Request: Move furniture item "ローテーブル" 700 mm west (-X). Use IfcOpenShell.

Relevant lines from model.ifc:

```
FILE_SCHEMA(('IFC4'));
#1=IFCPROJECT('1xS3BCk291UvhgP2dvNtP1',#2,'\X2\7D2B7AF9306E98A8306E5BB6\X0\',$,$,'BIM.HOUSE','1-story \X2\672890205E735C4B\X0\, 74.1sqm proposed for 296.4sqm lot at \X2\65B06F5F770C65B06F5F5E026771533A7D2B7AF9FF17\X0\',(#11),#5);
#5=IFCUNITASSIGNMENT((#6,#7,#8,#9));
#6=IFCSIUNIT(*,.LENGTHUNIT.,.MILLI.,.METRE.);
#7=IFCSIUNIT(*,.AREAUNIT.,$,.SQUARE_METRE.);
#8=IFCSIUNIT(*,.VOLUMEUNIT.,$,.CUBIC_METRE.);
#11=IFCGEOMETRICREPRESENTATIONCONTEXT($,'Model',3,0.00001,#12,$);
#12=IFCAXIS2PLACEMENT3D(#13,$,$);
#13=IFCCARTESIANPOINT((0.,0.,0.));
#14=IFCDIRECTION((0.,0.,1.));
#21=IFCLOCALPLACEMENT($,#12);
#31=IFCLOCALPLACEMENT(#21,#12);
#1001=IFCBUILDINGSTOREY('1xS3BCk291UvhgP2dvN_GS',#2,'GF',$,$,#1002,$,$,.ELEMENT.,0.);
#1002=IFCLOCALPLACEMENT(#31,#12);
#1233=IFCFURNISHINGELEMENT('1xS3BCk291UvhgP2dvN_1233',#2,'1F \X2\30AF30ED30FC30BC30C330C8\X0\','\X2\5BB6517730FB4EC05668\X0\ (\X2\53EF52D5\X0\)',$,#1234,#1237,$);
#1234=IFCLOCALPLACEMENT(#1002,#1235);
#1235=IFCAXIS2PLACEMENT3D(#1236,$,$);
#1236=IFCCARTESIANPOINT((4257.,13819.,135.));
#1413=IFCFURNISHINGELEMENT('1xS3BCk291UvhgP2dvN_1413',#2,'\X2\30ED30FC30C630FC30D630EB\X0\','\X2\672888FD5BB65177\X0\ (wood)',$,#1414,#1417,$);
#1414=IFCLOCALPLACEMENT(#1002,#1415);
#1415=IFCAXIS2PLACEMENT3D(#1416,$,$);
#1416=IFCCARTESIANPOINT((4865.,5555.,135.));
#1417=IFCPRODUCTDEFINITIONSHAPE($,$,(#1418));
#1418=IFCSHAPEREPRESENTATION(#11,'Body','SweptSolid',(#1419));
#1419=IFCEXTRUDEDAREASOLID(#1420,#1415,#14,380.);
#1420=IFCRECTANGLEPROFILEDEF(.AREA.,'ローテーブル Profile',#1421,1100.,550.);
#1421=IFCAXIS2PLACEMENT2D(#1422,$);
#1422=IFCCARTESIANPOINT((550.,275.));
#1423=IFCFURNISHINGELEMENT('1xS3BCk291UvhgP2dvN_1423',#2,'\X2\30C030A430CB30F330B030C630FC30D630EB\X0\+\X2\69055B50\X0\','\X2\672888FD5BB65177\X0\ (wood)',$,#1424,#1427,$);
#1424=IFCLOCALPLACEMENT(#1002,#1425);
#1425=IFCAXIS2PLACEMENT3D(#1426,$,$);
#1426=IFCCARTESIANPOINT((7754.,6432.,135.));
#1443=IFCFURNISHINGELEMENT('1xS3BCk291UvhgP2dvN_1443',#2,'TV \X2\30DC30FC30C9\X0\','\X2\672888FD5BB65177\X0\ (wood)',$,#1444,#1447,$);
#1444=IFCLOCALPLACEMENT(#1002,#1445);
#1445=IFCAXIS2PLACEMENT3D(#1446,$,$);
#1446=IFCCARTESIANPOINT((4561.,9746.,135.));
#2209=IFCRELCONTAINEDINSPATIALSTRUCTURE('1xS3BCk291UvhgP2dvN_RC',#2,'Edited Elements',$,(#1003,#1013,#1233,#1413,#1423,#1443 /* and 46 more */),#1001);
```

```python
import ifcopenshell
import ifcopenshell.api.geometry
import ifcopenshell.util.placement
import ifcopenshell.util.unit

model = ifcopenshell.open("model.ifc")
unit_scale = ifcopenshell.util.unit.calculate_unit_scale(model)

item = model.by_guid("1xS3BCk291UvhgP2dvN_1413")
matrix = ifcopenshell.util.placement.get_local_placement(item.ObjectPlacement)
matrix[0, 3] -= 0.7 / unit_scale
ifcopenshell.api.geometry.edit_object_placement(model, product=item, matrix=matrix, is_si=False)

print(ifcopenshell.util.placement.get_local_placement(item.ObjectPlacement).round(3) + 0.0)

model.write("model-out.ifc")
```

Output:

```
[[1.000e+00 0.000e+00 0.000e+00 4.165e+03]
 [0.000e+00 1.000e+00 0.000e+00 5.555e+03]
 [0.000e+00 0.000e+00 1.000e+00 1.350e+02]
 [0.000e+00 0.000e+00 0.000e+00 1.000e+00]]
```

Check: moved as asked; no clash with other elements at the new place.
